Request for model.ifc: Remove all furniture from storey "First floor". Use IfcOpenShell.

First a look at what the model holds.

```python
import ifcopenshell
import ifcopenshell.util.element

model = ifcopenshell.open("model.ifc")
print(model.schema)
storey = next(s for s in model.by_type("IfcBuildingStorey") if s.Name == "First floor")
furniture = [e for e in ifcopenshell.util.element.get_decomposition(storey) if e.is_a("IfcFurnishingElement")]
seen = {}
for e in furniture:
    element_type = ifcopenshell.util.element.get_type(e)
    name = element_type.Name if element_type not in (None, e) else None
    seen[name] = seen.get(name, 0) + 1
for name, count in sorted(seen.items(), key=str):
    print(count, "x", name)
```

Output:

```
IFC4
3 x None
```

```python
import ifcopenshell
import ifcopenshell.api.root
import ifcopenshell.util.element

model = ifcopenshell.open("model.ifc")

storey = next(s for s in model.by_type("IfcBuildingStorey") if s.Name == "First floor")
furniture = [e for e in ifcopenshell.util.element.get_decomposition(storey) if e.is_a("IfcFurnishingElement")]

for e in furniture:
    ifcopenshell.api.root.remove_product(model, product=e)
print(len(furniture), "removed")

model.write("model_rev.ifc")
```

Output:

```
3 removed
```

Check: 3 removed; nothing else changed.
